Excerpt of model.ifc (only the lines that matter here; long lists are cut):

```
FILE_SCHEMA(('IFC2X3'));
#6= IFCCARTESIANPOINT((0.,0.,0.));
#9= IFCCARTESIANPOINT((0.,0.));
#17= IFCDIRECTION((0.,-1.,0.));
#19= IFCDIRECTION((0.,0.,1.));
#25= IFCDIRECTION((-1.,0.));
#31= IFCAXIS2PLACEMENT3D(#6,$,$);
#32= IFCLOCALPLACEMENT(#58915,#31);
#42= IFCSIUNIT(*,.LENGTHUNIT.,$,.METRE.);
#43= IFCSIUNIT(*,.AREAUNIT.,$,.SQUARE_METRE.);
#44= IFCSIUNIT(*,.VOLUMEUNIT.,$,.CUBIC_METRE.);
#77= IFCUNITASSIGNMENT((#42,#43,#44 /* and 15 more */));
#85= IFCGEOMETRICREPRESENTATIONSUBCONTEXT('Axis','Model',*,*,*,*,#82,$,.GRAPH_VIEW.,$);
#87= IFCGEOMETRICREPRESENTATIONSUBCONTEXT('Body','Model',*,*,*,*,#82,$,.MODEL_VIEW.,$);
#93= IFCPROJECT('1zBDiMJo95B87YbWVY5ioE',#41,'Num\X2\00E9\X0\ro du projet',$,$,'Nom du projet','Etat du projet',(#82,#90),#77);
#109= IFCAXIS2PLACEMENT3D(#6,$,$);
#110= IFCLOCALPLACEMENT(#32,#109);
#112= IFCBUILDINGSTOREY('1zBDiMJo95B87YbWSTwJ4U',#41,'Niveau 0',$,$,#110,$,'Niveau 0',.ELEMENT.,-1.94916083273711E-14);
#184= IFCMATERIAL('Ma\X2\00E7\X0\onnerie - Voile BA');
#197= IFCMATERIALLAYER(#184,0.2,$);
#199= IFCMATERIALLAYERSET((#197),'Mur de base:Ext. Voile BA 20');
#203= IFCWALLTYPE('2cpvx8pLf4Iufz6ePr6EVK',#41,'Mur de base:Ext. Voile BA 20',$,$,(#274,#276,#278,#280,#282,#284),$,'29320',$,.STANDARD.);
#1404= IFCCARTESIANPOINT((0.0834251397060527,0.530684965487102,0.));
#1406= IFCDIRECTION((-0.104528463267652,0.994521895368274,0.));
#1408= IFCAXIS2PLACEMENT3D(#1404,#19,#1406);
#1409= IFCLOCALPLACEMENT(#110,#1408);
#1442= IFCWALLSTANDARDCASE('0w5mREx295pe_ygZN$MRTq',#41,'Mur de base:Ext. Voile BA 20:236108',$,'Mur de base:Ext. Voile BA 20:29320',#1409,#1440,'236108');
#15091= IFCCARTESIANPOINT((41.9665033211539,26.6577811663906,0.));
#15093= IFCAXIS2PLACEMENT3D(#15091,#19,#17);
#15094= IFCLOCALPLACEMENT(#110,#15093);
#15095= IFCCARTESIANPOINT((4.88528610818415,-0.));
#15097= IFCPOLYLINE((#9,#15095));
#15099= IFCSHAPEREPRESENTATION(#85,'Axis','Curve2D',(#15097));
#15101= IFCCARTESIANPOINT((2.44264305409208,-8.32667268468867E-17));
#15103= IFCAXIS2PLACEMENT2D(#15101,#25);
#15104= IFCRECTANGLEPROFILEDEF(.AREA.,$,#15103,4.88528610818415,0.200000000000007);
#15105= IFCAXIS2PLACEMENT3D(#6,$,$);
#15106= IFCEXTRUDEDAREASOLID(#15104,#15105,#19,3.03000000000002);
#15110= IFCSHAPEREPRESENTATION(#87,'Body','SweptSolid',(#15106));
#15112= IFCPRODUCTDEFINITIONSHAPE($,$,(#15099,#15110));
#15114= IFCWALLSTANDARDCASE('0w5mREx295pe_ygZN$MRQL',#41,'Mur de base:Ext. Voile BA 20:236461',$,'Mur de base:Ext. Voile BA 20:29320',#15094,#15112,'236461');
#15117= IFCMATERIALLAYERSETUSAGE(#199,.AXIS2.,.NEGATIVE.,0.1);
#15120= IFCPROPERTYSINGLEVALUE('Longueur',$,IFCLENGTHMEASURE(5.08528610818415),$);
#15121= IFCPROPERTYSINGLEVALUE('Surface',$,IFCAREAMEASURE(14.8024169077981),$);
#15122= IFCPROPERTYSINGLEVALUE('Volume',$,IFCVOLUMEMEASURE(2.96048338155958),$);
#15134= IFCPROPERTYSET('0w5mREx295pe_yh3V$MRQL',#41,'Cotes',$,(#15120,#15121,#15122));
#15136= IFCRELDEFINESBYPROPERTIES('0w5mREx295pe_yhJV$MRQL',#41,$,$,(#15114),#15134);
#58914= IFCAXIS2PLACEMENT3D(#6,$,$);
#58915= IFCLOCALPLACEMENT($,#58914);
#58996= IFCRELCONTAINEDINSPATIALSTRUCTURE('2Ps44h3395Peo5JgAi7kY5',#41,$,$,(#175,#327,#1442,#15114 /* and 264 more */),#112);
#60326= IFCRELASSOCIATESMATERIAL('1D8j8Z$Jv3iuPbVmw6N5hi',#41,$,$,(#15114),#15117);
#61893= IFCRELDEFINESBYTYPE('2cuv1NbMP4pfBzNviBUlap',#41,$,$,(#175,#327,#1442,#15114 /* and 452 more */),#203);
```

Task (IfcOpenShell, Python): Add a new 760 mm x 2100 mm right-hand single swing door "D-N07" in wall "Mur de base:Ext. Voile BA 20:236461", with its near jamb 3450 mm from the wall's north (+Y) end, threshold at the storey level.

```python
import numpy as np
import ifcopenshell
import ifcopenshell.api.feature
import ifcopenshell.api.geometry
import ifcopenshell.api.pset
import ifcopenshell.api.root
import ifcopenshell.api.spatial
import ifcopenshell.api.type
import ifcopenshell.geom
import ifcopenshell.util.element
import ifcopenshell.util.placement
import ifcopenshell.util.representation
import ifcopenshell.util.shape
import ifcopenshell.util.unit

model = ifcopenshell.open("model.ifc")
unit_scale = ifcopenshell.util.unit.calculate_unit_scale(model)
area_scale = ifcopenshell.util.unit.calculate_unit_scale(model, "AREAUNIT")
volume_scale = ifcopenshell.util.unit.calculate_unit_scale(model, "VOLUMEUNIT")
settings = ifcopenshell.geom.settings()


def volume(element):
    """Net volume in cubic metres, openings subtracted."""
    shape = ifcopenshell.geom.create_shape(settings, element)
    return ifcopenshell.util.shape.get_volume(shape.geometry)


wall = model.by_guid("0w5mREx295pe_ygZN$MRQL")
storey = ifcopenshell.util.element.get_container(wall, ifc_class="IfcBuildingStorey")
context = ifcopenshell.util.representation.get_context(model, "Model", "Body", "MODEL_VIEW")
before = volume(wall)

width, height, from_end, sill = 0.76, 2.1, 3.45, 0.0  # metres

# The wall runs along its own X axis, and the end named is its -X end.
wall_shape = ifcopenshell.geom.create_shape(settings, wall)
x, y, z = ifcopenshell.util.shape.get_vertices(wall_shape.geometry).T
start = x.min() + from_end
face, thickness = float(y.min()), float(y.max() - y.min())
wall_matrix = ifcopenshell.util.placement.get_local_placement(wall.ObjectPlacement)
level = ifcopenshell.util.placement.get_local_placement(storey.ObjectPlacement)[2, 3]


def in_wall(x, y):
    """Placement at x, y metres in the wall's axes, at sill height."""
    matrix = wall_matrix.copy()
    matrix[:, 3] = wall_matrix @ np.array([x / unit_scale, y / unit_scale, 0.0, 1.0])
    matrix[2, 3] = level + sill / unit_scale
    return matrix


# Opening: a box that overshoots both wall faces by 50 mm.
opening = ifcopenshell.api.root.create_entity(model, ifc_class="IfcOpeningElement")
box = ifcopenshell.api.geometry.add_wall_representation(
    model, context=context, length=width, height=height, thickness=thickness + 0.1
)
ifcopenshell.api.geometry.assign_representation(model, product=opening, representation=box)
ifcopenshell.api.geometry.edit_object_placement(model, product=opening, matrix=in_wall(start, face - 0.05), is_si=False)
ifcopenshell.api.feature.add_feature(model, feature=opening, element=wall)

door = ifcopenshell.api.root.create_entity(model, ifc_class="IfcDoor", name="D-N07")
door.OverallWidth, door.OverallHeight = width / unit_scale, height / unit_scale
body = ifcopenshell.api.geometry.add_door_representation(
    model,
    context=context,
    overall_width=door.OverallWidth,
    overall_height=door.OverallHeight,
    operation_type="SINGLE_SWING_RIGHT",
    lining_properties={"LiningDepth": thickness / unit_scale, "ThresholdDepth": thickness / unit_scale},
)
ifcopenshell.api.geometry.assign_representation(model, product=door, representation=body)
ifcopenshell.api.spatial.assign_container(model, products=[door], relating_structure=storey)
fills = ifcopenshell.api.feature.add_filling(model, opening=opening, element=door)
fills.OwnerHistory = door.OwnerHistory  # required in IFC2X3

# IFC2X3 keeps the operation on the door style.
style = ifcopenshell.api.root.create_entity(model, ifc_class="IfcDoorStyle", name="D-N07")
style.OperationType, style.ConstructionType = "SINGLE_SWING_RIGHT", "NOTDEFINED"
style.ParameterTakesPrecedence = style.Sizeable = False
ifcopenshell.api.type.assign_type(model, related_objects=[door], relating_type=style)

# The lining spans the wall, so the door starts at the wall face.
ifcopenshell.api.geometry.edit_object_placement(model, product=door, matrix=in_wall(start, face), is_si=False)

after = volume(wall)

# Update the wall's stored quantities.
pset = model.by_id(ifcopenshell.util.element.get_pset(wall, "Cotes", should_inherit=False)["id"])
ifcopenshell.api.pset.edit_pset(model, pset=pset, properties={
    "Surface": model.create_entity("IfcAreaMeasure", after / thickness / area_scale),
    "Volume": model.create_entity("IfcVolumeMeasure", after / volume_scale),
})

print(f"wall volume {before:.3f} -> {after:.3f} m3")

model.write("model_rev.ifc")
```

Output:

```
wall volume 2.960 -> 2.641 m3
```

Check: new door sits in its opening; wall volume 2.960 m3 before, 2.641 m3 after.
